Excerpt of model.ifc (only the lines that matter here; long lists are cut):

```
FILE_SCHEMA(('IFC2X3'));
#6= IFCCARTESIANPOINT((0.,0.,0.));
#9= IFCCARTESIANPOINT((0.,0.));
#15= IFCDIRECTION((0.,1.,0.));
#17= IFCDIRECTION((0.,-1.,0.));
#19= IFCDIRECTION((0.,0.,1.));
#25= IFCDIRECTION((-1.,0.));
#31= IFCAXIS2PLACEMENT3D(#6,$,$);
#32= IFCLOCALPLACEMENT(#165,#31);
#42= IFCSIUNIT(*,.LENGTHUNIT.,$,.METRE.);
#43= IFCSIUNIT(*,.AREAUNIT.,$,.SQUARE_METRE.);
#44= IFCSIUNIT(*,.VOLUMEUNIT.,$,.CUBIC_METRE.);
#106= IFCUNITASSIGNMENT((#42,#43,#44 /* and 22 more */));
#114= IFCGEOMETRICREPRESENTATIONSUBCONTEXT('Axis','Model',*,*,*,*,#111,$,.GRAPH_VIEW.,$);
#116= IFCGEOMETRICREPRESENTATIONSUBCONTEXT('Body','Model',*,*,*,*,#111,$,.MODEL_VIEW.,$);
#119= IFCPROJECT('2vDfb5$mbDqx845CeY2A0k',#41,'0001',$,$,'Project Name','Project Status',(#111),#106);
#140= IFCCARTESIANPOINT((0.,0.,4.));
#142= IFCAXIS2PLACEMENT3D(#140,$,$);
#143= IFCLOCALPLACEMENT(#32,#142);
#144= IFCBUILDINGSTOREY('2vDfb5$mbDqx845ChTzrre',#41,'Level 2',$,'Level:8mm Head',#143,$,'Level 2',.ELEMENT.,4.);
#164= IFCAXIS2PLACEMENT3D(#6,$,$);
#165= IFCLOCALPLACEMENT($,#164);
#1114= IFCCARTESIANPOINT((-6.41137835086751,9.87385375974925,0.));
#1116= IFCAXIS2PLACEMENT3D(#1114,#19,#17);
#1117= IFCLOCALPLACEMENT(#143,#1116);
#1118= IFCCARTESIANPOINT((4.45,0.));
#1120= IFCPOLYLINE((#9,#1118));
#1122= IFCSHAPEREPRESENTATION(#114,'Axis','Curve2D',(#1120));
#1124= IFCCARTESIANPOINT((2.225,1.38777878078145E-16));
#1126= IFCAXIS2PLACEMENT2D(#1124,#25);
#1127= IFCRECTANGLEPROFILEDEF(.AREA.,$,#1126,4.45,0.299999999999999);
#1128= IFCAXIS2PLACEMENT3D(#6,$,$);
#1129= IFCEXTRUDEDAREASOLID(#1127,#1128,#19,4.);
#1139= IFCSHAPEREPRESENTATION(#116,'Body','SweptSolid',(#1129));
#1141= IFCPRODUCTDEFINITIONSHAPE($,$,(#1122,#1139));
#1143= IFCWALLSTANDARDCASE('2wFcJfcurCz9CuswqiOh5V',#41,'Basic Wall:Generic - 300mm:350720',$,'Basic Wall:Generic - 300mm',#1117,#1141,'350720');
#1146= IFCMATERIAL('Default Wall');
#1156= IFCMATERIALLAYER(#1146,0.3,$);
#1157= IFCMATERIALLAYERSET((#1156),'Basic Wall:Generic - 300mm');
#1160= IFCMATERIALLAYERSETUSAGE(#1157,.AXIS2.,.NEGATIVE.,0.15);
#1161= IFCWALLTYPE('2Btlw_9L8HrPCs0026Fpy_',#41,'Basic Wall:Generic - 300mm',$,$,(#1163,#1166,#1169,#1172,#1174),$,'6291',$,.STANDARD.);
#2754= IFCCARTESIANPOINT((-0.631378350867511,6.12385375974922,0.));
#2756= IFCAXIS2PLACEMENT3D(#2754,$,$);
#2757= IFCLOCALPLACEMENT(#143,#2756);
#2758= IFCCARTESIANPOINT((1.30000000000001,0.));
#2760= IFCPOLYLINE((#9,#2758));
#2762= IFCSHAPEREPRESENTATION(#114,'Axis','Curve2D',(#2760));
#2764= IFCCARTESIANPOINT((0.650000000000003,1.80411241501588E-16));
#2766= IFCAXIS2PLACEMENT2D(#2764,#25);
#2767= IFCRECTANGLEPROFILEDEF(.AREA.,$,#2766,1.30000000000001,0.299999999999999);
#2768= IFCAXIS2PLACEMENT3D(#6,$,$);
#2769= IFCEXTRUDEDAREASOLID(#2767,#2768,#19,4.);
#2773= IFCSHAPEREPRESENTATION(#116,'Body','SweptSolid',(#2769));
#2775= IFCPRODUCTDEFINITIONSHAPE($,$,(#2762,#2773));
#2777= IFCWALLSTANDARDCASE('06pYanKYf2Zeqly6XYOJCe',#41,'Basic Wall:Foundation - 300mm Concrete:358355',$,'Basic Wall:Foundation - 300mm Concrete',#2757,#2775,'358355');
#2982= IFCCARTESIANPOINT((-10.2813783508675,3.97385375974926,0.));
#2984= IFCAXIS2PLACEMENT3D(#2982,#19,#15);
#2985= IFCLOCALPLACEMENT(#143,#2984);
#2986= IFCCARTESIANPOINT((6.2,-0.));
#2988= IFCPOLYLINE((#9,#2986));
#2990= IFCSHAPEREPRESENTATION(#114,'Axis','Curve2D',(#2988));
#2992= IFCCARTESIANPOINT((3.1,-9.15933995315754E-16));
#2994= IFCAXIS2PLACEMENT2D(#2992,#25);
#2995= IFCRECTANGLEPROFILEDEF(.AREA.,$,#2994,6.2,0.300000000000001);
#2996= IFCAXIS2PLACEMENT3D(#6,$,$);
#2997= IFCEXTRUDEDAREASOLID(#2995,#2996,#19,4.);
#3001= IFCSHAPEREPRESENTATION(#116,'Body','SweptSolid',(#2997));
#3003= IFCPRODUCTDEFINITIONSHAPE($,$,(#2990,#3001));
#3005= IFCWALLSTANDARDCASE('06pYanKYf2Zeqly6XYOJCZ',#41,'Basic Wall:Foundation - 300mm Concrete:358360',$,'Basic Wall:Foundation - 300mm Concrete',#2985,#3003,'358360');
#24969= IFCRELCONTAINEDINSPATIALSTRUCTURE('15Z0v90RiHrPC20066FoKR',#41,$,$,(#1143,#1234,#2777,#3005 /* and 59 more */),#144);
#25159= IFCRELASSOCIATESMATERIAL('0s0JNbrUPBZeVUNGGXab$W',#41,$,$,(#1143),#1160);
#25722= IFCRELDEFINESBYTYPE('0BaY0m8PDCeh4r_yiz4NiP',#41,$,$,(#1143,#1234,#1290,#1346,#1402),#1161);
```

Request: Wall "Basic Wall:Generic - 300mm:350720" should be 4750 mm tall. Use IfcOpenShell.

```python
import ifcopenshell
import ifcopenshell.geom
import ifcopenshell.util.representation
import ifcopenshell.util.shape
import ifcopenshell.util.unit

model = ifcopenshell.open("model.ifc")
unit_scale = ifcopenshell.util.unit.calculate_unit_scale(model)
settings = ifcopenshell.geom.settings()


def volume(element):
    """Net volume in cubic metres, openings subtracted."""
    shape = ifcopenshell.geom.create_shape(settings, element)
    return ifcopenshell.util.shape.get_volume(shape.geometry)


wall = model.by_guid("2wFcJfcurCz9CuswqiOh5V")
before = volume(wall)

body = ifcopenshell.util.representation.get_representation(wall, "Model", "Body")
solid = body.Items[0]
old_height = solid.Depth
solid.Depth = 4.75 / unit_scale
after = volume(wall)

print(f"height {old_height:g} -> {solid.Depth:g}, volume {before:.3f} -> {after:.3f} m3")

model.write("model_edited.ifc")
```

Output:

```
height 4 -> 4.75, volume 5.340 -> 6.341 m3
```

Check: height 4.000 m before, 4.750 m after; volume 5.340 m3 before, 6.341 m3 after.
